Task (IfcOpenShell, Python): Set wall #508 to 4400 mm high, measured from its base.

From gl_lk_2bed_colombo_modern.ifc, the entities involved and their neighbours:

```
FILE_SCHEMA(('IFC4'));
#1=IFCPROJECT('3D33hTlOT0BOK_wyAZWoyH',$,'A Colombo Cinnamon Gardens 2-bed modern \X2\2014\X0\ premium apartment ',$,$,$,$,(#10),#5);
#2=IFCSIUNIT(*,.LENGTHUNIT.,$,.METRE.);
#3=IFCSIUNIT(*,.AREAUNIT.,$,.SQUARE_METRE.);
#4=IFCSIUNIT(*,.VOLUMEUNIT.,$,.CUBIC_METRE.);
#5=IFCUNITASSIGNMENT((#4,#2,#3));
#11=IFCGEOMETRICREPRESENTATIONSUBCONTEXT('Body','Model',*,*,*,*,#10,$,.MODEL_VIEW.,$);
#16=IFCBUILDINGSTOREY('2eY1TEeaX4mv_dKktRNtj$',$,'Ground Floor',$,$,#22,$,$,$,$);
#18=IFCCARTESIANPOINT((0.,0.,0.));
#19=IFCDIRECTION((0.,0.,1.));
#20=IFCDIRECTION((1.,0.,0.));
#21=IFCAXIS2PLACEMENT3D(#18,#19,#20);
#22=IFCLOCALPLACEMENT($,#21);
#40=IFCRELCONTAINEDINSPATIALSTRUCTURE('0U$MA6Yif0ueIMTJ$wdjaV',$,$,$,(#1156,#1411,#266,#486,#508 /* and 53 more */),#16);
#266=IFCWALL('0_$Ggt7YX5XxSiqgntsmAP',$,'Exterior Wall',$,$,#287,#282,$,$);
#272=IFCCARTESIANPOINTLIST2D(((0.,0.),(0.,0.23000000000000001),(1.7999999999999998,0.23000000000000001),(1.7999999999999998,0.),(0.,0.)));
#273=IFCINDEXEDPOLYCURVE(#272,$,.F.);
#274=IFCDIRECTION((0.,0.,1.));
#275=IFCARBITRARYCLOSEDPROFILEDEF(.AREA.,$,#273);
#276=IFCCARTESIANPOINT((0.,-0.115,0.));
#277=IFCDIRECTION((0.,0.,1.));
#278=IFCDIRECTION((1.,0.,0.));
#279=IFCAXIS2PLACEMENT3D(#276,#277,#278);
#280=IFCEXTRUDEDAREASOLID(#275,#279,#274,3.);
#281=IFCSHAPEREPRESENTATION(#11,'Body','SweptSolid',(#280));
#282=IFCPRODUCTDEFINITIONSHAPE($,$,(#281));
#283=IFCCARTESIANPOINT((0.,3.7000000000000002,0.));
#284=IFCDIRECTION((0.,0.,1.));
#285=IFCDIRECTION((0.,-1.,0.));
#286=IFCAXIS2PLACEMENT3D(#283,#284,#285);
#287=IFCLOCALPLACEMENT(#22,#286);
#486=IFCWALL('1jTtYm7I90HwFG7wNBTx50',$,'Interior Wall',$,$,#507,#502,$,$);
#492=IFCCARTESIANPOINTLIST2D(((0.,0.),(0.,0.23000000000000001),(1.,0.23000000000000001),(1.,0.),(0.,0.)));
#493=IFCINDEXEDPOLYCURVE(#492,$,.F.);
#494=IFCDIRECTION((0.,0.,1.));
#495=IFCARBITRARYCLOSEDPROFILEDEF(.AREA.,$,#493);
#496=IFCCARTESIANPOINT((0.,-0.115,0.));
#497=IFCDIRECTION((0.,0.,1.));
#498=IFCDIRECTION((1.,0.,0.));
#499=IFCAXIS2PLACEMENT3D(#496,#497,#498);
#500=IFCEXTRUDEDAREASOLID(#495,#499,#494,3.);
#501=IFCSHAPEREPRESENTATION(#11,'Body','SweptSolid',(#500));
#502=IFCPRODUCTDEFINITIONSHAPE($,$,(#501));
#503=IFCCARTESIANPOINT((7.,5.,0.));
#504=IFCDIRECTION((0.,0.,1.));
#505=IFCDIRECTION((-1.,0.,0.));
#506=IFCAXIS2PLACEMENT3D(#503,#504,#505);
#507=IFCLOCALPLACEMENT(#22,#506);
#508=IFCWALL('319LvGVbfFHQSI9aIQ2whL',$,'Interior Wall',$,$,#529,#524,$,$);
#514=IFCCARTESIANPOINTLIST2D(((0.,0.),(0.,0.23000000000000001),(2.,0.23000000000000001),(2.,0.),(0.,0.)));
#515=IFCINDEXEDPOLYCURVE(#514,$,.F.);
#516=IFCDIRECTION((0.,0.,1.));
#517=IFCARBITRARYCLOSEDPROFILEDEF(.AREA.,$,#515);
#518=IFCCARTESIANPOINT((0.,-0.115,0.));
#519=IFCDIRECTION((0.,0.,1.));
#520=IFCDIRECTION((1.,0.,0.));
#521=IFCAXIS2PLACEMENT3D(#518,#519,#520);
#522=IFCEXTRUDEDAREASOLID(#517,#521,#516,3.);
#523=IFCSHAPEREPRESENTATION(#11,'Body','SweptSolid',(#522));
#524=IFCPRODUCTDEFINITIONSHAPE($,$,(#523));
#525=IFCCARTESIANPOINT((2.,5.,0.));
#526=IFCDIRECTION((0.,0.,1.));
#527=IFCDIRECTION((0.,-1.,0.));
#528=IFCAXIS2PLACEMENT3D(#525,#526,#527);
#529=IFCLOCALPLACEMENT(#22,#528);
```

```python
import ifcopenshell
import ifcopenshell.geom
import ifcopenshell.util.representation
import ifcopenshell.util.shape
import ifcopenshell.util.unit

model = ifcopenshell.open("gl_lk_2bed_colombo_modern.ifc")
unit_scale = ifcopenshell.util.unit.calculate_unit_scale(model)
settings = ifcopenshell.geom.settings()


def volume(element):
    """Net volume in cubic metres, openings subtracted."""
    shape = ifcopenshell.geom.create_shape(settings, element)
    return ifcopenshell.util.shape.get_volume(shape.geometry)


wall = model.by_guid("319LvGVbfFHQSI9aIQ2whL")
before = volume(wall)

body = ifcopenshell.util.representation.get_representation(wall, "Model", "Body")
solid = body.Items[0]
old_height = solid.Depth
solid.Depth = 4.4 / unit_scale
after = volume(wall)

print(f"height {old_height:g} -> {solid.Depth:g}, volume {before:.3f} -> {after:.3f} m3")

model.write("gl_lk_2bed_colombo_modern-out.ifc")
```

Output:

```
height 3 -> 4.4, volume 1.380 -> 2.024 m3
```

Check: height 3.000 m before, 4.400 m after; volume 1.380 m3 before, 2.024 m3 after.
